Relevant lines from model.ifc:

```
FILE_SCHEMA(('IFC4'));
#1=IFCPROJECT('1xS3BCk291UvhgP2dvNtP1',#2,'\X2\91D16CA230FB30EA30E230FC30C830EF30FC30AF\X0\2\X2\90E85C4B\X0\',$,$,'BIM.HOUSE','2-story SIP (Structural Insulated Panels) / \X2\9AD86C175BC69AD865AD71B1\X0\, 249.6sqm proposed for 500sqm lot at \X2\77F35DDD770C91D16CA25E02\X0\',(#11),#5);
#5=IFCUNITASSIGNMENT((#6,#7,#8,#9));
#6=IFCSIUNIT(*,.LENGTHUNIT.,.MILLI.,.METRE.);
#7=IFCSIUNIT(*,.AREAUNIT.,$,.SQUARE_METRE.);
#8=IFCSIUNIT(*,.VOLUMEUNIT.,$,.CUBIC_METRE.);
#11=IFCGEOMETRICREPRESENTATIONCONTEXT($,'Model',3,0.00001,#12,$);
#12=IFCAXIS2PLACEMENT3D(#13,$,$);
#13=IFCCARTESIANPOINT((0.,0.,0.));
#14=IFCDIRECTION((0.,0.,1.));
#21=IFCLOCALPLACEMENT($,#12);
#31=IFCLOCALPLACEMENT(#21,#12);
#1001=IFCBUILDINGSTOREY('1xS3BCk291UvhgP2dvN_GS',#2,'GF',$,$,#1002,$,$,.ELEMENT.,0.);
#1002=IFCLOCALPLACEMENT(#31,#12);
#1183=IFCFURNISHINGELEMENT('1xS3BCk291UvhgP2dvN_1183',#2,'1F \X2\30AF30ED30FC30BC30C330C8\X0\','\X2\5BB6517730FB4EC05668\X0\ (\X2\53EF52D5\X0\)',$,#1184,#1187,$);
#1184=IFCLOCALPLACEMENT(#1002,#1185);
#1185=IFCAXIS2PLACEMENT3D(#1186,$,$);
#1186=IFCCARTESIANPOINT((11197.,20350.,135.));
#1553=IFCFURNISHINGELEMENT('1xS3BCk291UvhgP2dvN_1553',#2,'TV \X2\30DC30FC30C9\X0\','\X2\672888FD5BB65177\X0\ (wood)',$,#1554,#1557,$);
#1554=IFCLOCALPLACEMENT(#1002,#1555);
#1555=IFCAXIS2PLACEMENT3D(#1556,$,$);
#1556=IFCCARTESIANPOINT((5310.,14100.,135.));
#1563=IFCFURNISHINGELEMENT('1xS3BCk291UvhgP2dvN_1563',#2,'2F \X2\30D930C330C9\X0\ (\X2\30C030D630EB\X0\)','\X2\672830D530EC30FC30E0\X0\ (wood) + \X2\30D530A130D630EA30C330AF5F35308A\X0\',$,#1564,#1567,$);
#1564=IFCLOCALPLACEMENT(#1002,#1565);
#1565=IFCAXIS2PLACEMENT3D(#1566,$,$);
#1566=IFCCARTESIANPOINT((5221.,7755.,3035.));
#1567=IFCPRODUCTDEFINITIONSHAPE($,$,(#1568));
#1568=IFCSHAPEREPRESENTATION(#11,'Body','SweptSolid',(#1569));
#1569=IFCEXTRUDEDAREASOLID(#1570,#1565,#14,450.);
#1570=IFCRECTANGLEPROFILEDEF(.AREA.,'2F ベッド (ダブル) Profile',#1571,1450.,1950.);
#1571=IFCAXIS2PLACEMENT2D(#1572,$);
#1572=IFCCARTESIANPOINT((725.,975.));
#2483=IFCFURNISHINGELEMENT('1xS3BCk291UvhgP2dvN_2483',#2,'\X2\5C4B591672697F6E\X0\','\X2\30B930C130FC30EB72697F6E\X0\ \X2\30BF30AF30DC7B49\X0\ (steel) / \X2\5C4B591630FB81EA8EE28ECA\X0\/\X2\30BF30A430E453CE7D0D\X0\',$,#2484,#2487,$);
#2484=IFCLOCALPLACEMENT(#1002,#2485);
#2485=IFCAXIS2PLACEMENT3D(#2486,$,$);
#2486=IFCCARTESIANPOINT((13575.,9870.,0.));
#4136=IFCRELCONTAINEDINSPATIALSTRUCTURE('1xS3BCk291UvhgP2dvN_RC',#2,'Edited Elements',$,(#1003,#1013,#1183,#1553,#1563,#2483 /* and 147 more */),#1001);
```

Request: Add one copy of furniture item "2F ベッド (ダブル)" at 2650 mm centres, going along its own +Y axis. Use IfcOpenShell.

```python
import ifcopenshell
import ifcopenshell.api.geometry
import ifcopenshell.api.root
import ifcopenshell.util.element
import ifcopenshell.util.placement
import ifcopenshell.util.unit

model = ifcopenshell.open("model.ifc")
unit_scale = ifcopenshell.util.unit.calculate_unit_scale(model)


def reuse_history(source, copy):
    """copy_class also copies each property set's owner history, people and application; keep the originals."""
    for rel in copy.IsDefinedBy:
        if rel.is_a("IfcRelDefinesByProperties") and (history := rel.RelatingPropertyDefinition.OwnerHistory):
            rel.RelatingPropertyDefinition.OwnerHistory = source.OwnerHistory
            ifcopenshell.util.element.remove_deep2(model, history)


source = model.by_guid("1xS3BCk291UvhgP2dvN_1563")
base = ifcopenshell.util.placement.get_local_placement(source.ObjectPlacement)
step = base[:3, 1] * 2.65 / unit_scale

for i in range(1, 2):
    copy = ifcopenshell.api.root.copy_class(model, product=source)
    copy.Representation = ifcopenshell.util.element.copy_deep(
        model, source.Representation, exclude=["IfcGeometricRepresentationContext", "IfcRepresentationMap"]
    )
    reuse_history(source, copy)
    matrix = base.copy()
    matrix[:3, 3] += i * step
    print("added at", matrix[:3, 3].round(3) + 0.0)
    ifcopenshell.api.geometry.edit_object_placement(model, product=copy, matrix=matrix, is_si=False)

model.write("model_rev.ifc")
```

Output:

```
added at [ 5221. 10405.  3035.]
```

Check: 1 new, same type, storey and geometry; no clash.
